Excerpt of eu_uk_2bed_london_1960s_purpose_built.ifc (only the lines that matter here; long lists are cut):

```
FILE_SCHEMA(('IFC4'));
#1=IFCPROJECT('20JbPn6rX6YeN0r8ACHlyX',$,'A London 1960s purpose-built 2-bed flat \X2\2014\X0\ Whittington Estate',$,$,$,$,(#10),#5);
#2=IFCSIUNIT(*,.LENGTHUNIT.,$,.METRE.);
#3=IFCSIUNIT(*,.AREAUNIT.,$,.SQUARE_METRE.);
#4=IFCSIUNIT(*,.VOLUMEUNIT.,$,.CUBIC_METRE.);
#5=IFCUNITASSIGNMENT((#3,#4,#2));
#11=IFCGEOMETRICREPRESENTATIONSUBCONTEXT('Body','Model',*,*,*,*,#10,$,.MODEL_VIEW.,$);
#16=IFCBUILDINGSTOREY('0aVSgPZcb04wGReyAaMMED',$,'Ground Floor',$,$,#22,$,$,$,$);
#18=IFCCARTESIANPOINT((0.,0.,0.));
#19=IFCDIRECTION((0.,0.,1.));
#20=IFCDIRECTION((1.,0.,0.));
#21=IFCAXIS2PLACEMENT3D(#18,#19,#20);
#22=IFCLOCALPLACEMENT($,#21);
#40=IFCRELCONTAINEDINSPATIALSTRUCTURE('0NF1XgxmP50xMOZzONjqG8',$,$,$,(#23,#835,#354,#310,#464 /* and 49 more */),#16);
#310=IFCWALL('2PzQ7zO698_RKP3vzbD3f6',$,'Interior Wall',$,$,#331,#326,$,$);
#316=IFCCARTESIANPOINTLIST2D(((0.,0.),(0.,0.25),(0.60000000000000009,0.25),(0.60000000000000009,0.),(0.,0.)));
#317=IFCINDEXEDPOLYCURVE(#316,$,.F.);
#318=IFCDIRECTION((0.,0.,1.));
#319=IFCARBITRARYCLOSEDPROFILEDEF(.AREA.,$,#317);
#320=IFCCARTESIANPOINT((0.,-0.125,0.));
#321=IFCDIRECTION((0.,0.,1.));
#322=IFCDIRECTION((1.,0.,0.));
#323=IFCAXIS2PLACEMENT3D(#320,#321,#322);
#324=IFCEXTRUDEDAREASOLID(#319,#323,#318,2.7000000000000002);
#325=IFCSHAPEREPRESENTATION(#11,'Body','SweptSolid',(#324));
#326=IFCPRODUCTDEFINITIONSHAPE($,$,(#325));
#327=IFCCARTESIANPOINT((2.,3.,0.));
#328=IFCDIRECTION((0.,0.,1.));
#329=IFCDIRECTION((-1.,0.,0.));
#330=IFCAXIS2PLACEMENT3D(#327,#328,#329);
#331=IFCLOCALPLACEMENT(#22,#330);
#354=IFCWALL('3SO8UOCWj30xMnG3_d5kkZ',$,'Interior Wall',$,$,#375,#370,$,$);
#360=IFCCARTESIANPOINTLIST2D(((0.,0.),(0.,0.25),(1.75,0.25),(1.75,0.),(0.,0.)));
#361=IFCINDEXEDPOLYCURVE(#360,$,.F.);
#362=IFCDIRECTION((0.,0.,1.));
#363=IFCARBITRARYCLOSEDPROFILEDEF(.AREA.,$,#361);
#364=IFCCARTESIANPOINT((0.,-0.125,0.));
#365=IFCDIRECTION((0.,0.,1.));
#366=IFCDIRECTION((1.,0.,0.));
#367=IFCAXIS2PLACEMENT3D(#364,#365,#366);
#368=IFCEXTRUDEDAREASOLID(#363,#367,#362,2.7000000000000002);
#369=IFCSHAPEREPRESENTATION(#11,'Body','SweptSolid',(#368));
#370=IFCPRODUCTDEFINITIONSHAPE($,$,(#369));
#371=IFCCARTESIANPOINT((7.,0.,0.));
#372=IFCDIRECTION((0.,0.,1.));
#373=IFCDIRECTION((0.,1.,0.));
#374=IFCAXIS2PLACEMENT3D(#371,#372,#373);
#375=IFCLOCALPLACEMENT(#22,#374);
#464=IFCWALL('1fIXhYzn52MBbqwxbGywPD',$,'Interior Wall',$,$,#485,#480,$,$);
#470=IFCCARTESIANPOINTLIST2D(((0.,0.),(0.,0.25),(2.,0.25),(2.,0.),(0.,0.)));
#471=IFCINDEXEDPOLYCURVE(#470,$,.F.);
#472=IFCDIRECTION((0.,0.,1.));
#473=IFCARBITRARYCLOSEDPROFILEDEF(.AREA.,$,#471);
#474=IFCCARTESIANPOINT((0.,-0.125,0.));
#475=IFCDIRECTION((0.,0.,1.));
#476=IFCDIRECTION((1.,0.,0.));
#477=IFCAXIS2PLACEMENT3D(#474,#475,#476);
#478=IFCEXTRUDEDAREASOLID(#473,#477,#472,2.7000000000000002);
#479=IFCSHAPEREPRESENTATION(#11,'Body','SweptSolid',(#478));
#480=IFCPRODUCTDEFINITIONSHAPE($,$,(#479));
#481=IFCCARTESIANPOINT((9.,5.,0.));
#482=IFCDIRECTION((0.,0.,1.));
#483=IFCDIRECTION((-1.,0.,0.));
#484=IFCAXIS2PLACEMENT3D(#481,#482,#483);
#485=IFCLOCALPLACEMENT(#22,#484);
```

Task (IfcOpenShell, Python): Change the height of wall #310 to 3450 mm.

```python
import ifcopenshell
import ifcopenshell.geom
import ifcopenshell.util.representation
import ifcopenshell.util.shape
import ifcopenshell.util.unit

model = ifcopenshell.open("eu_uk_2bed_london_1960s_purpose_built.ifc")
unit_scale = ifcopenshell.util.unit.calculate_unit_scale(model)
settings = ifcopenshell.geom.settings()


def volume(element):
    """Net volume in cubic metres, openings subtracted."""
    shape = ifcopenshell.geom.create_shape(settings, element)
    return ifcopenshell.util.shape.get_volume(shape.geometry)


wall = model.by_guid("2PzQ7zO698_RKP3vzbD3f6")
before = volume(wall)

body = ifcopenshell.util.representation.get_representation(wall, "Model", "Body")
solid = body.Items[0]
old_height = solid.Depth
solid.Depth = 3.45 / unit_scale
after = volume(wall)

print(f"height {old_height:g} -> {solid.Depth:g}, volume {before:.3f} -> {after:.3f} m3")

model.write("eu_uk_2bed_london_1960s_purpose_built-out.ifc")
```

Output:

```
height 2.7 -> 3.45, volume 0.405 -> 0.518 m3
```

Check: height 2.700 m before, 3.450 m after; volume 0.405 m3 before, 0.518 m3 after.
